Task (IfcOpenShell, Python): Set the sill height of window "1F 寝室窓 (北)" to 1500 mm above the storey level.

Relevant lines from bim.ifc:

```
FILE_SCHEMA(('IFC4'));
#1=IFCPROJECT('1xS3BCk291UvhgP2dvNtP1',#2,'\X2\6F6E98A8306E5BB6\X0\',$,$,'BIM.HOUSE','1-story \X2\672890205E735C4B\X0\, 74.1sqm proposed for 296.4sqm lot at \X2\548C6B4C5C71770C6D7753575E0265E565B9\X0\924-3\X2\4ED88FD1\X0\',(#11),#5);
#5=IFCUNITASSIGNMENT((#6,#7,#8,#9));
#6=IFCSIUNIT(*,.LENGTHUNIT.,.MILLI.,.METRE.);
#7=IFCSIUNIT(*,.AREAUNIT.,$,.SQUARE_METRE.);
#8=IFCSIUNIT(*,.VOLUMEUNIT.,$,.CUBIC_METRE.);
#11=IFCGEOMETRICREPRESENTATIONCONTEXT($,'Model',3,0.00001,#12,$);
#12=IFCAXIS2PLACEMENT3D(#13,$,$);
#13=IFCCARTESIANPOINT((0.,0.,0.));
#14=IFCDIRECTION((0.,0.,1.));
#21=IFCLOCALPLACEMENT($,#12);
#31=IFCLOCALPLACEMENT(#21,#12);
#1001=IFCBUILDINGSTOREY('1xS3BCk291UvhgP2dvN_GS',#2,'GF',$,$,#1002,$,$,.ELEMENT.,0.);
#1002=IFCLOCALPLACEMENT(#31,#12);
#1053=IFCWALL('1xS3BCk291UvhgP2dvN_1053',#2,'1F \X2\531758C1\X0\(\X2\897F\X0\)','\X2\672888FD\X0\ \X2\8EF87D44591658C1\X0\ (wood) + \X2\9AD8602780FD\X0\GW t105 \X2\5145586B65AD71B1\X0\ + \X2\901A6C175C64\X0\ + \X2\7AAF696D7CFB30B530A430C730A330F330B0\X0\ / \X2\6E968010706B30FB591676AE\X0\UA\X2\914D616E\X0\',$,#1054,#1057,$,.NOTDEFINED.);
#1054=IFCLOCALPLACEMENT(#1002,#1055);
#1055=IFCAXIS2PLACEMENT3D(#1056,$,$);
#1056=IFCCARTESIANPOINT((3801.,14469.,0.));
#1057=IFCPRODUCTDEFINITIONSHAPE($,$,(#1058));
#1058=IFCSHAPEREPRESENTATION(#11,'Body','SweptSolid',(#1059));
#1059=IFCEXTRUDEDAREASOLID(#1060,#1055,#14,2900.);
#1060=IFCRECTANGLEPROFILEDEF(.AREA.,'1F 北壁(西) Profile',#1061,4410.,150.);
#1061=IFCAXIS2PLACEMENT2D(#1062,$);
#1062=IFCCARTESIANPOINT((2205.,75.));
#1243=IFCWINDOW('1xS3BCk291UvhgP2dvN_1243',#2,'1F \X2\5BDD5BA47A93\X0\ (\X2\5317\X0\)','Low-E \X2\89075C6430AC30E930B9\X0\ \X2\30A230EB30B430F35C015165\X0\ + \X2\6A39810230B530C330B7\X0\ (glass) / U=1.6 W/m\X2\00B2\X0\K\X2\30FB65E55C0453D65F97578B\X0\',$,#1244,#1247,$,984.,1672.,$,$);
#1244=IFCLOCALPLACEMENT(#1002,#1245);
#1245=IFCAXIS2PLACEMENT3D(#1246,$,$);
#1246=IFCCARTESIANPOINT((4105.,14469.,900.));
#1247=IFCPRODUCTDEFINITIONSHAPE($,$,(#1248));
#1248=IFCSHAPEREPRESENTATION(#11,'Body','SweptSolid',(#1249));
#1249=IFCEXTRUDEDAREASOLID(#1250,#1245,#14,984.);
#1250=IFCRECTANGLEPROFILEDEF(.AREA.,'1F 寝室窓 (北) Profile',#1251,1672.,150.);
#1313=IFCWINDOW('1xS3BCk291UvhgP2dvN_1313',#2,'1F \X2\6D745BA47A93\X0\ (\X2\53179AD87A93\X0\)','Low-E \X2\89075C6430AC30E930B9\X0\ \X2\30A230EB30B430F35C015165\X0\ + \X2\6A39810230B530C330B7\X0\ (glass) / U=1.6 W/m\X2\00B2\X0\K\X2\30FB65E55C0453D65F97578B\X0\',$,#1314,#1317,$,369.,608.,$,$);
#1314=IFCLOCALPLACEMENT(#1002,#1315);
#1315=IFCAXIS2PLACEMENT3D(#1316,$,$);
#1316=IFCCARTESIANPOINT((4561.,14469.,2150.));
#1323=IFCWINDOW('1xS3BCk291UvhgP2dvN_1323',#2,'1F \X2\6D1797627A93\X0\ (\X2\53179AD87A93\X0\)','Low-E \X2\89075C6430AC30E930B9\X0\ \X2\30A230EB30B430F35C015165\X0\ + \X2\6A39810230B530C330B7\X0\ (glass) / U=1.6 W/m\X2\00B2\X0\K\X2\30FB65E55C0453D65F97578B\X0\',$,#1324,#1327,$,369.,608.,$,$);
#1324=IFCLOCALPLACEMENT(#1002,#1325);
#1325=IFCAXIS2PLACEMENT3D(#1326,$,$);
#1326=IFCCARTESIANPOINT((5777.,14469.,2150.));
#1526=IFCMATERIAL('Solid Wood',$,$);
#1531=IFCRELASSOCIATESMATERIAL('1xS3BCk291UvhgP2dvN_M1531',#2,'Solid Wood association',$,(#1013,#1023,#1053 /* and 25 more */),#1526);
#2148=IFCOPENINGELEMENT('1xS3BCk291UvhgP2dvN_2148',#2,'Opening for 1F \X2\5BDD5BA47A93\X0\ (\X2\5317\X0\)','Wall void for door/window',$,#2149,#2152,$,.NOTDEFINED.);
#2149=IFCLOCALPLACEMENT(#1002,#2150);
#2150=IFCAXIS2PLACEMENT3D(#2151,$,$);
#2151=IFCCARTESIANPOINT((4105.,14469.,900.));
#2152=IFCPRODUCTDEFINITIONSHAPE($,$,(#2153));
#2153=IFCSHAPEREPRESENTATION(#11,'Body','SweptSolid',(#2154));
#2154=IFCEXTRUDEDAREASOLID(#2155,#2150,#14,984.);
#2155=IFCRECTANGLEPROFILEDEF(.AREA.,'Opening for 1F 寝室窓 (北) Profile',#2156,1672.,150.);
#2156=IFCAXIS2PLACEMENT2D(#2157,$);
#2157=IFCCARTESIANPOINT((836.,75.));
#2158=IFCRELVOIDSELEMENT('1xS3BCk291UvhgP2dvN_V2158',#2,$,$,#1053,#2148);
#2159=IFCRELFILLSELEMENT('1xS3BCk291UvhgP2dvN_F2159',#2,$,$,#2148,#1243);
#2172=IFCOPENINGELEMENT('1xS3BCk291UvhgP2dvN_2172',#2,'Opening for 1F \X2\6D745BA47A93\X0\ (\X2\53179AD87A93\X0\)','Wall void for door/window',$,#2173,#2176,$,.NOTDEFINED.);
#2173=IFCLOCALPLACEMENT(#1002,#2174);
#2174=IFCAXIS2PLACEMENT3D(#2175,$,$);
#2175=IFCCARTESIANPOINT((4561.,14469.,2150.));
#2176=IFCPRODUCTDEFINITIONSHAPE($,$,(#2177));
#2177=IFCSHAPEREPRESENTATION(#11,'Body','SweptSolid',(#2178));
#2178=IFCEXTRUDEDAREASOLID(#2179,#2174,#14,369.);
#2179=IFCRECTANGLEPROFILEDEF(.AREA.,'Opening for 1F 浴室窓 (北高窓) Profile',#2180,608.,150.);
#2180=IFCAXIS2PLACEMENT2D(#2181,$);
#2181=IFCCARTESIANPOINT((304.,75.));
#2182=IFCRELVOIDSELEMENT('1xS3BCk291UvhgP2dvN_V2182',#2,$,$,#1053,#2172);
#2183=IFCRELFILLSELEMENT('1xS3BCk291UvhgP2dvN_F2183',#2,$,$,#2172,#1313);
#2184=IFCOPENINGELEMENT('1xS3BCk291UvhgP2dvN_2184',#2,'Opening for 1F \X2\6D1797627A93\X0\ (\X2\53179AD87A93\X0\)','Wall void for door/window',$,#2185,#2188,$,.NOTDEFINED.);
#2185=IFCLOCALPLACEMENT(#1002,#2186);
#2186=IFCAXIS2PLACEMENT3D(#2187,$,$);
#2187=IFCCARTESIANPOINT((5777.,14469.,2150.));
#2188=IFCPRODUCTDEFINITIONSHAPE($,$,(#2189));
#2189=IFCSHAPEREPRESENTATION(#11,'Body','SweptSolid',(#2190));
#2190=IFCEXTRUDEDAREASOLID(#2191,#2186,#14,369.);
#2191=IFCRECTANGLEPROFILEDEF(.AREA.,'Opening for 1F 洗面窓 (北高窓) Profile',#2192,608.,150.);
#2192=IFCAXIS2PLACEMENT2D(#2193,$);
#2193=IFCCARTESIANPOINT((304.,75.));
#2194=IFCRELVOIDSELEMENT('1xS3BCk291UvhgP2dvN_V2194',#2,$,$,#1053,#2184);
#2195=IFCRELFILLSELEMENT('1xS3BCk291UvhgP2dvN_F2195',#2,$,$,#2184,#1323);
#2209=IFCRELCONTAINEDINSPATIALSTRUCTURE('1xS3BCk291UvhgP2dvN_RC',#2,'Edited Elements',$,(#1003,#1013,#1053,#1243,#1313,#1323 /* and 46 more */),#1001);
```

```python
import numpy as np
import ifcopenshell
import ifcopenshell.api.geometry
import ifcopenshell.geom
import ifcopenshell.util.element
import ifcopenshell.util.placement
import ifcopenshell.util.shape
import ifcopenshell.util.unit

model = ifcopenshell.open("bim.ifc")
unit_scale = ifcopenshell.util.unit.calculate_unit_scale(model)

window = model.by_guid("1xS3BCk291UvhgP2dvN_1243")
opening = window.FillsVoids[0].RelatingOpeningElement
storey = ifcopenshell.util.element.get_container(window, ifc_class="IfcBuildingStorey")
level = ifcopenshell.util.placement.get_local_placement(storey.ObjectPlacement)[2, 3]

# The opening's origin need not be at the sill, so measure its lowest point.
shape = ifcopenshell.geom.create_shape(ifcopenshell.geom.settings(), opening)
bottom = ifcopenshell.util.shape.get_shape_bottom_elevation(shape, shape.geometry) / unit_scale
dz = level + 1.5 / unit_scale - bottom

shift = np.array([0.0, 0.0, dz])
# The window is not placed relative to its opening, so move both.
for product in (opening, window):
    matrix = ifcopenshell.util.placement.get_local_placement(product.ObjectPlacement)
    matrix[:3, 3] += shift
    ifcopenshell.api.geometry.edit_object_placement(model, product=product, matrix=matrix, is_si=False)

print(f"moved by {dz * unit_scale:+.3f} m")

model.write("bim_updated.ifc")
```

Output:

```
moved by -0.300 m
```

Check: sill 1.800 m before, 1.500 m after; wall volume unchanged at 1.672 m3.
